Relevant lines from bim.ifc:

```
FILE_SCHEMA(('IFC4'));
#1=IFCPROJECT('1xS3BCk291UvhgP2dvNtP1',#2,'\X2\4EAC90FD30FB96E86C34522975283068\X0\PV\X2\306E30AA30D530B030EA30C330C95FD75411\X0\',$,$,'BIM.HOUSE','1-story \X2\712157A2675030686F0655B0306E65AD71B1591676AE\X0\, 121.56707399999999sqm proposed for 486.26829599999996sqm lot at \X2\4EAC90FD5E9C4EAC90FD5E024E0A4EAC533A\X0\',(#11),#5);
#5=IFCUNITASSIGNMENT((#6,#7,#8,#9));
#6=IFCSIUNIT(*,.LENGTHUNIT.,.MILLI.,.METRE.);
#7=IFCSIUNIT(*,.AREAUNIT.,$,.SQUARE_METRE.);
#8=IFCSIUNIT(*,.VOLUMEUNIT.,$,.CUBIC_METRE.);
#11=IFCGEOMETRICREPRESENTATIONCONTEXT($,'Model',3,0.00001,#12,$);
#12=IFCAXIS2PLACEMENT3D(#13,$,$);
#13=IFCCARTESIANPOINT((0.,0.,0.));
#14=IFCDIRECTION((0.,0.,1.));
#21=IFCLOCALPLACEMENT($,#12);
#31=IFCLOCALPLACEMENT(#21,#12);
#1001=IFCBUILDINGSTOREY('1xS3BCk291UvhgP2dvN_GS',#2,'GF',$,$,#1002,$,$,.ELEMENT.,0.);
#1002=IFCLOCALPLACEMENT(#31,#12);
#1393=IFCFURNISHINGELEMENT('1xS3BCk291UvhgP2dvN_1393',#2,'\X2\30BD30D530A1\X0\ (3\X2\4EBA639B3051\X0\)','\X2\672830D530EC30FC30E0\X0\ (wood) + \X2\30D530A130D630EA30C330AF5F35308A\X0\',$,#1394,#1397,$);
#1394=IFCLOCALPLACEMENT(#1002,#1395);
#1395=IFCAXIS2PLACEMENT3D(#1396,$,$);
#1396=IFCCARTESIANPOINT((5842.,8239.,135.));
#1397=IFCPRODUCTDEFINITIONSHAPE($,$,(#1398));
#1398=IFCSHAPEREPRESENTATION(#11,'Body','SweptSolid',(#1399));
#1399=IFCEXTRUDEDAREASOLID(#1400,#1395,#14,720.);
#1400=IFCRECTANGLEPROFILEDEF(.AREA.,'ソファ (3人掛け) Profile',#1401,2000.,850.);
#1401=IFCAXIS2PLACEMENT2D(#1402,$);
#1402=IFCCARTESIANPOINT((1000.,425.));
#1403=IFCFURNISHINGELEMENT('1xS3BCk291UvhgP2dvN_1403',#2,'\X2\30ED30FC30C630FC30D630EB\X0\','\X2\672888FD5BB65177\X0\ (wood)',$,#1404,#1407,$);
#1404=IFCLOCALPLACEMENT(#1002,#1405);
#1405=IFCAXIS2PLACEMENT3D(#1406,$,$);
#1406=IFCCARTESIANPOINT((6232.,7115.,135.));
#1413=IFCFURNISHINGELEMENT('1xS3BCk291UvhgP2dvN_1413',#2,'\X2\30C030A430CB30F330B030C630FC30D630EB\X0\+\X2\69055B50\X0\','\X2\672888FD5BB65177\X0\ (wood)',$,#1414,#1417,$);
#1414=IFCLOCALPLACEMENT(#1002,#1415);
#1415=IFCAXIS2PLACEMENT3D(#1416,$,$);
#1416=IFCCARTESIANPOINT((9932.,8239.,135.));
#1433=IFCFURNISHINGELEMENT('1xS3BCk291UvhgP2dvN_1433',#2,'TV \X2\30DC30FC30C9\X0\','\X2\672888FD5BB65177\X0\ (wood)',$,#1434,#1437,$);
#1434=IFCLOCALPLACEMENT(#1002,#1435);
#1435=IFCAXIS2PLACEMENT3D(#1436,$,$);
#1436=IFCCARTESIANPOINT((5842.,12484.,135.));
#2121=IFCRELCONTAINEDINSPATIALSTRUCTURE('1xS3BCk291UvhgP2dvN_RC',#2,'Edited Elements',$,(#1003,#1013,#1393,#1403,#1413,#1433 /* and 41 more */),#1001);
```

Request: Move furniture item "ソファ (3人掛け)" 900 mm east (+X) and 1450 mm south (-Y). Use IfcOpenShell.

```python
import ifcopenshell
import ifcopenshell.api.geometry
import ifcopenshell.util.placement

model = ifcopenshell.open("bim.ifc")

item = model.by_guid("1xS3BCk291UvhgP2dvN_1393")
matrix = ifcopenshell.util.placement.get_local_placement(item.ObjectPlacement)
matrix[0, 3] += 900.0
matrix[1, 3] -= 1450.0
ifcopenshell.api.geometry.edit_object_placement(model, product=item, matrix=matrix, is_si=False)

print(ifcopenshell.util.placement.get_local_placement(item.ObjectPlacement).round(3) + 0.0)

model.write("bim_rev.ifc")
```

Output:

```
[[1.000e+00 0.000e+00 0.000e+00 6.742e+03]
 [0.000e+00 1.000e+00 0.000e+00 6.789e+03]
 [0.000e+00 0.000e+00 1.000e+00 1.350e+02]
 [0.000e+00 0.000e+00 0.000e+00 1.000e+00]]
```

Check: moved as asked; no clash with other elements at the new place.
